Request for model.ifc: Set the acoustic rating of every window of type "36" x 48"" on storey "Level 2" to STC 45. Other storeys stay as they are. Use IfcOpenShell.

First a look at what the model holds.

```python
import ifcopenshell
import ifcopenshell.util.element

model = ifcopenshell.open("model.ifc")
print(model.schema)
storey = next(s for s in model.by_type("IfcBuildingStorey") if s.Name == "Level 2")
windows = [e for e in ifcopenshell.util.element.get_decomposition(storey) if e.is_a("IfcWindow")]
seen = {}
for e in windows:
    element_type = ifcopenshell.util.element.get_type(e)
    key = (element_type.Name if element_type != e and element_type else None, ifcopenshell.util.element.get_pset(e, "Pset_WindowCommon", "AcousticRating"))
    seen[key] = seen.get(key, 0) + 1
for (name, value), count in sorted(seen.items(), key=str):
    print(count, "x", name, "|", value)
```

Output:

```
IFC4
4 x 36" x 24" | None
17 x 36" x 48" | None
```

```python
import ifcopenshell
import ifcopenshell.api.pset
import ifcopenshell.util.element

model = ifcopenshell.open("model.ifc")

storey = next(s for s in model.by_type("IfcBuildingStorey") if s.Name == "Level 2")
windows = [e for e in ifcopenshell.util.element.get_decomposition(storey) if e.is_a("IfcWindow")]

count = 0
for e in windows:
    element_type = ifcopenshell.util.element.get_type(e)
    if element_type in (None, e) or element_type.Name != '36" x 48"':
        continue
    # add_pset returns the element's existing set when there is one.
    pset = ifcopenshell.api.pset.add_pset(model, product=e, name="Pset_WindowCommon")
    ifcopenshell.api.pset.edit_pset(model, pset=pset, properties={"AcousticRating": "STC 45"})
    count += 1

print(count, "windows updated")

model.write("model_edited.ifc")
```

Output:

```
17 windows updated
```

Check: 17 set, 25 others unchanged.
